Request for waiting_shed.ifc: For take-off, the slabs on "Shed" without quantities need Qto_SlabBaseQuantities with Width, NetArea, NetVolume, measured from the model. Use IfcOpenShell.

First a look at what the model holds.

```python
import ifcopenshell
import ifcopenshell.util.element
import ifcopenshell.util.unit

model = ifcopenshell.open("waiting_shed.ifc")
print(model.schema)
for unit_type in ("LENGTHUNIT", "AREAUNIT", "VOLUMEUNIT"):
    print(unit_type, ifcopenshell.util.unit.calculate_unit_scale(model, unit_type))
storey = next(s for s in model.by_type("IfcBuildingStorey") if s.Name == "Shed")
slabs = [e for e in ifcopenshell.util.element.get_decomposition(storey) if e.is_a("IfcSlab")]
for e in sorted(slabs, key=lambda e: e.id()):
    print(e.id(), e.is_a(), e.Name, list(ifcopenshell.util.element.get_psets(e, qtos_only=True)), sep=" | ")
```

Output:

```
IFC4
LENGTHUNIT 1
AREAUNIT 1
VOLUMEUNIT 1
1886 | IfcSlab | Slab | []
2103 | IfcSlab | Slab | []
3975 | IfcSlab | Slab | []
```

```python
import ifcopenshell
import ifcopenshell.api.pset
import ifcopenshell.geom
import ifcopenshell.util.element
import ifcopenshell.util.shape
import ifcopenshell.util.unit

model = ifcopenshell.open("waiting_shed.ifc")
unit_scale = ifcopenshell.util.unit.calculate_unit_scale(model)
area_scale = ifcopenshell.util.unit.calculate_unit_scale(model, "AREAUNIT")
volume_scale = ifcopenshell.util.unit.calculate_unit_scale(model, "VOLUMEUNIT")
settings = ifcopenshell.geom.settings()

storey = next(s for s in model.by_type("IfcBuildingStorey") if s.Name == "Shed")
slabs = [e for e in ifcopenshell.util.element.get_decomposition(storey) if e.is_a("IfcSlab")]

for e in sorted(slabs, key=lambda e: e.id()):
    if ifcopenshell.util.element.get_psets(e, qtos_only=True, should_inherit=False):
        continue
    # Geometry comes back in metres, in the element's own axes.
    shape = ifcopenshell.geom.create_shape(settings, e)
    values = {
        "Width": ifcopenshell.util.shape.get_z(shape.geometry) / unit_scale,
        "NetArea": ifcopenshell.util.shape.get_footprint_area(shape.geometry) / area_scale,
        "NetVolume": ifcopenshell.util.shape.get_volume(shape.geometry) / volume_scale,
    }
    qto = ifcopenshell.api.pset.add_qto(model, product=e, name="Qto_SlabBaseQuantities")
    ifcopenshell.api.pset.edit_qto(model, qto=qto, properties=values)
    print(e.id(), {k: round(v, 3) for k, v in values.items()})

model.write("waiting_shed_edited.ifc")
```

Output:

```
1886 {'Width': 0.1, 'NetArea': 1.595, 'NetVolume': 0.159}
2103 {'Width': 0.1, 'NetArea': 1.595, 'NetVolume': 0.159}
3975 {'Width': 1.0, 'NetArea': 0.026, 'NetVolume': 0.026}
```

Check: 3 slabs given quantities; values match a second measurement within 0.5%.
